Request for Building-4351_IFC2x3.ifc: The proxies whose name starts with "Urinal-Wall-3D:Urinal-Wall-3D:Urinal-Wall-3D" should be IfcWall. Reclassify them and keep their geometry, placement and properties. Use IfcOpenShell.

First a look at what the model holds.

```python
import re

import ifcopenshell

model = ifcopenshell.open("Building-4351_IFC2x3.ifc")
print(model.schema)
seen = {}
for e in model.by_type("IfcBuildingElementProxy"):
    name = re.sub(r":\d+(:\d+)?$", "", e.Name or "")  # drop the element id that some exporters append
    seen[name] = seen.get(name, 0) + 1
for name, count in sorted(seen.items()):
    print(count, "x", name)
```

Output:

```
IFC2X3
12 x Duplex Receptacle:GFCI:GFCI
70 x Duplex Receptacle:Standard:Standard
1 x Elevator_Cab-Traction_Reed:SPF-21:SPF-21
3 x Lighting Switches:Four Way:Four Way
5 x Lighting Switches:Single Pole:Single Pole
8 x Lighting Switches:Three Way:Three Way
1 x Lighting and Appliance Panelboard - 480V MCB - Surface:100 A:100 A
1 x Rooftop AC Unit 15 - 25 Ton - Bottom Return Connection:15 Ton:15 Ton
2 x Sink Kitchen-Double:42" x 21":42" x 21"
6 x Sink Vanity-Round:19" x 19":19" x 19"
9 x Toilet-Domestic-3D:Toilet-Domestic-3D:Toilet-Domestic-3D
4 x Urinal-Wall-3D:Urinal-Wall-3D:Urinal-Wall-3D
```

```python
import ifcopenshell
import ifcopenshell.api.root

model = ifcopenshell.open("Building-4351_IFC2x3.ifc")

proxies = [e.id() for e in model.by_type("IfcBuildingElementProxy") if (e.Name or "").startswith("Urinal-Wall-3D:Urinal-Wall-3D:Urinal-Wall-3D")]
for step_id in proxies:
    proxy = model.by_id(step_id)
    ifcopenshell.api.root.reassign_class(model, product=proxy, ifc_class="IfcWall")

print(sum(model.by_id(i).is_a("IfcWall") for i in proxies), "reclassified")

model.write("Building-4351_IFC2x3_updated.ifc")
```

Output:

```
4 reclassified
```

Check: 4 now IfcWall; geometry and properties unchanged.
